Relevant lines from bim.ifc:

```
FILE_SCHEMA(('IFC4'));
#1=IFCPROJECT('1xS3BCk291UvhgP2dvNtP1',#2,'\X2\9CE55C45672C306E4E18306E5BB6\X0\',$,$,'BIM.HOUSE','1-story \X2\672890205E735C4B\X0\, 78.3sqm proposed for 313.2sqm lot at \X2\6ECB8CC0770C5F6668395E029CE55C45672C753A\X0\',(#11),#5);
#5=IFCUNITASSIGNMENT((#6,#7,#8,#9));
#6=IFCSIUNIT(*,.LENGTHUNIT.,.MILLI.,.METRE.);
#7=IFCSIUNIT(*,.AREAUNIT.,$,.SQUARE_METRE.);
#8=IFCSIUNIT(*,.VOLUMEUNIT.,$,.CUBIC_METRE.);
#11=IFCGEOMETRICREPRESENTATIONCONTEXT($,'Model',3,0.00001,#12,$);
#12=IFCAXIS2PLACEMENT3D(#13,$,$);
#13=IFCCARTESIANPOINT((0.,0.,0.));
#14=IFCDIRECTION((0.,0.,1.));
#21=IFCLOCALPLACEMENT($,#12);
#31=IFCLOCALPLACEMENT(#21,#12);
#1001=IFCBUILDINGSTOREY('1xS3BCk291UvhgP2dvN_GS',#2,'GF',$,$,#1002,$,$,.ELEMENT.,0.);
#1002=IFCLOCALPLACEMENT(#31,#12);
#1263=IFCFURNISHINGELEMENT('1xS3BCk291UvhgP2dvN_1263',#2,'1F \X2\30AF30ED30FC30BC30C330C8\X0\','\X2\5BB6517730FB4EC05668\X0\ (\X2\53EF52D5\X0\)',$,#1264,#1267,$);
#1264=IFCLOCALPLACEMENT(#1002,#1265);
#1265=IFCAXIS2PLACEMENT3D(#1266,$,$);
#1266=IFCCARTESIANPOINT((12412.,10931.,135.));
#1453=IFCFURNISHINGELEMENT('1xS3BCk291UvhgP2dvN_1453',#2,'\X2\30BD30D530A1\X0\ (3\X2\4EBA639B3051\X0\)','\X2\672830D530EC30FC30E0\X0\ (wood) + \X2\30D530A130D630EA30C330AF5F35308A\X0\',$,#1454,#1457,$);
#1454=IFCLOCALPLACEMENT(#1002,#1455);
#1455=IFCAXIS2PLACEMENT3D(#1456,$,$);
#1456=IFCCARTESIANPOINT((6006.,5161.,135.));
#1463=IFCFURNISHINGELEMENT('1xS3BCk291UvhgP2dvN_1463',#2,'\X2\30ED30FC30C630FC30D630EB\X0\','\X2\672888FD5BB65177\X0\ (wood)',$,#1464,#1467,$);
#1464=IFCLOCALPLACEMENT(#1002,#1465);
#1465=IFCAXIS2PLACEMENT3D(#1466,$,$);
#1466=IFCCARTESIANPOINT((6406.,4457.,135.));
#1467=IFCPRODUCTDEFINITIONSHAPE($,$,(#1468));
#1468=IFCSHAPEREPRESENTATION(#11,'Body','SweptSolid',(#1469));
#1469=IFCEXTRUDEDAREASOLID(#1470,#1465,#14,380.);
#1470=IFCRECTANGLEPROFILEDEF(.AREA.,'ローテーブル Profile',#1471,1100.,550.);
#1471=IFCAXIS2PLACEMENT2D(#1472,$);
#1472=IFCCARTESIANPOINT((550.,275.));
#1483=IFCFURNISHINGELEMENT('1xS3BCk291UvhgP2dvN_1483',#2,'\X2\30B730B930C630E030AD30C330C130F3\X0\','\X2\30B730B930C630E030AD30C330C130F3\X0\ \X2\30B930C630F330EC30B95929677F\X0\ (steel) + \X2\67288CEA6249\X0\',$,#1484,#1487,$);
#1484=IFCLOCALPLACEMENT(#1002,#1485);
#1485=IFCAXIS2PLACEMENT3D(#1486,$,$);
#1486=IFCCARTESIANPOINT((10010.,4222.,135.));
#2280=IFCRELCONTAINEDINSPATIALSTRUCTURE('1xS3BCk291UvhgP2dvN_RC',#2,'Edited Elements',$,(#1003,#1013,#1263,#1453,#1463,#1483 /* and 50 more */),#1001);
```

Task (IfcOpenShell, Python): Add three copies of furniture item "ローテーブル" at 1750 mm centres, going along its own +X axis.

```python
import ifcopenshell
import ifcopenshell.api.geometry
import ifcopenshell.api.root
import ifcopenshell.util.element
import ifcopenshell.util.placement
import ifcopenshell.util.unit

model = ifcopenshell.open("bim.ifc")
unit_scale = ifcopenshell.util.unit.calculate_unit_scale(model)


def reuse_history(source, copy):
    """copy_class also copies each property set's owner history, people and application; keep the originals."""
    for rel in copy.IsDefinedBy:
        if rel.is_a("IfcRelDefinesByProperties") and (history := rel.RelatingPropertyDefinition.OwnerHistory):
            rel.RelatingPropertyDefinition.OwnerHistory = source.OwnerHistory
            ifcopenshell.util.element.remove_deep2(model, history)


source = model.by_id(1463)
base = ifcopenshell.util.placement.get_local_placement(source.ObjectPlacement)
step = base[:3, 0] * 1.75 / unit_scale

for i in range(1, 4):
    copy = ifcopenshell.api.root.copy_class(model, product=source)
    copy.Representation = ifcopenshell.util.element.copy_deep(
        model, source.Representation, exclude=["IfcGeometricRepresentationContext", "IfcRepresentationMap"]
    )
    reuse_history(source, copy)
    matrix = base.copy()
    matrix[:3, 3] += i * step
    print("added at", matrix[:3, 3].round(3) + 0.0)
    ifcopenshell.api.geometry.edit_object_placement(model, product=copy, matrix=matrix, is_si=False)

model.write("bim_rev.ifc")
```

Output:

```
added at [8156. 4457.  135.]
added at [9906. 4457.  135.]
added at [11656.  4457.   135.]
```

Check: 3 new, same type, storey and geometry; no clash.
